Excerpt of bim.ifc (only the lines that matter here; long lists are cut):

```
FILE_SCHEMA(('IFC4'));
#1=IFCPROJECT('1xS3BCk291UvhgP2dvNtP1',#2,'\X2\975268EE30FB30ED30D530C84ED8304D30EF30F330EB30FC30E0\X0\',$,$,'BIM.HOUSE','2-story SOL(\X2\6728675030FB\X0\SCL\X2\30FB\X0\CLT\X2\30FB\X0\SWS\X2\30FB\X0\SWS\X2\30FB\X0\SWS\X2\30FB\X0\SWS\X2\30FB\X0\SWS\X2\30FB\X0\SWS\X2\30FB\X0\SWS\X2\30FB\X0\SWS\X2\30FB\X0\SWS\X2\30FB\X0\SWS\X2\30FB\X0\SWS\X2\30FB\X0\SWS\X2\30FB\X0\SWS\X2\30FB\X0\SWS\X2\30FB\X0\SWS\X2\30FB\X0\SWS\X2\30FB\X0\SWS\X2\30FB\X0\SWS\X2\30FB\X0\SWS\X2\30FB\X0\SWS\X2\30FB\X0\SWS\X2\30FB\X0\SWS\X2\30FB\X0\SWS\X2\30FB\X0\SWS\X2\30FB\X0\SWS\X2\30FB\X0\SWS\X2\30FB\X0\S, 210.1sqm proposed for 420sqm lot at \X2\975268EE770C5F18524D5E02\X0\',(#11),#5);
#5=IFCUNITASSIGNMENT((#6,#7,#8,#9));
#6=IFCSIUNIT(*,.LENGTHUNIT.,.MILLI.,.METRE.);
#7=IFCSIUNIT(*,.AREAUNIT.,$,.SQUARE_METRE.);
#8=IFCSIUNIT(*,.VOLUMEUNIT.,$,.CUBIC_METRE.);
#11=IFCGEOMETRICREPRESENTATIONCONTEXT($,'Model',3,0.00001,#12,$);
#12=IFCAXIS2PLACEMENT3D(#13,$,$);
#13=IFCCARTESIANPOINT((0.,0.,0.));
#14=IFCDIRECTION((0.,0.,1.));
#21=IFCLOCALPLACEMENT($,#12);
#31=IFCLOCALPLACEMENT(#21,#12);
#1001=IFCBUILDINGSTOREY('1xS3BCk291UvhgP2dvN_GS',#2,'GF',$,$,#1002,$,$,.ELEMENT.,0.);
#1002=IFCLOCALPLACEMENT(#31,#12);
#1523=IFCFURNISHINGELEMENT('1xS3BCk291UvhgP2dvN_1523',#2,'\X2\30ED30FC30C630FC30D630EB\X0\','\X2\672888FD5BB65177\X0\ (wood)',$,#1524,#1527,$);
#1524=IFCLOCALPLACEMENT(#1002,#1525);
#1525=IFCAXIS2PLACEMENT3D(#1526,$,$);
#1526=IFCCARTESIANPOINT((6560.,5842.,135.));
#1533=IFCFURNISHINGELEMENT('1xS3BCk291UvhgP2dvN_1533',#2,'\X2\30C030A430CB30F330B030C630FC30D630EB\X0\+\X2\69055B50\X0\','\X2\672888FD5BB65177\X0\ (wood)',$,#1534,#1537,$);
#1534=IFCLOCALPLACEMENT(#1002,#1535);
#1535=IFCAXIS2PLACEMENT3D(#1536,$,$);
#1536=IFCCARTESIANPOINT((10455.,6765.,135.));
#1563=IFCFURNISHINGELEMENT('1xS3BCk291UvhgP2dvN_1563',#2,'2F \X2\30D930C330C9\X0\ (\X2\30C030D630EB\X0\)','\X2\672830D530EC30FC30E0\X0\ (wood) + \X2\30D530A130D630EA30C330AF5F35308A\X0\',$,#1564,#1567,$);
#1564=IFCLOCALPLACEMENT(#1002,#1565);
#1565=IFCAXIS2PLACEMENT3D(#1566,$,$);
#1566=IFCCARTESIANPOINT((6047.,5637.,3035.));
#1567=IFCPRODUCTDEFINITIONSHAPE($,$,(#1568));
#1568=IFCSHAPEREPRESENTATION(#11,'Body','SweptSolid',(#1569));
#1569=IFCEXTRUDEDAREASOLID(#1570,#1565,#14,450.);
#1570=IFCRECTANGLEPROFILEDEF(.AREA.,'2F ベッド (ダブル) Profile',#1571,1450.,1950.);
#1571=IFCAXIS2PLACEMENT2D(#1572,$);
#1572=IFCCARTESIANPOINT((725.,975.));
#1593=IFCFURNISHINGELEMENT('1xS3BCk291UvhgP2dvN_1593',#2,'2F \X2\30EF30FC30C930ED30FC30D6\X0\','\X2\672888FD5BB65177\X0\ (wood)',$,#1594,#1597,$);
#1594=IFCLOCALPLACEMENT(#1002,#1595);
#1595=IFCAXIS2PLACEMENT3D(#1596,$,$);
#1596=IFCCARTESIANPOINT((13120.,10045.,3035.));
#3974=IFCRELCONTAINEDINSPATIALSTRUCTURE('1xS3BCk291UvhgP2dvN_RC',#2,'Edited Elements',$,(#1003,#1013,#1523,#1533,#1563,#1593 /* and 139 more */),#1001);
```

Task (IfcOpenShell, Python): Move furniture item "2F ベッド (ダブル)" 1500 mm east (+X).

```python
import ifcopenshell
import ifcopenshell.api.geometry
import ifcopenshell.util.placement

model = ifcopenshell.open("bim.ifc")

item = model.by_id(1563)
matrix = ifcopenshell.util.placement.get_local_placement(item.ObjectPlacement)
matrix[0, 3] += 1500.0
ifcopenshell.api.geometry.edit_object_placement(model, product=item, matrix=matrix, is_si=False)

print(ifcopenshell.util.placement.get_local_placement(item.ObjectPlacement).round(3) + 0.0)

model.write("bim_v2.ifc")
```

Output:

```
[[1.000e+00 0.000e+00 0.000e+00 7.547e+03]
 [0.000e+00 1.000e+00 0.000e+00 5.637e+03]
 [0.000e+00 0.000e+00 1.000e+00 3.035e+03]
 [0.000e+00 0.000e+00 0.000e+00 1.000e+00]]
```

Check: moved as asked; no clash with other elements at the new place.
